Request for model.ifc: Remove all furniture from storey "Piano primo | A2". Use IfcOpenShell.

First a look at what the model holds.

```python
import ifcopenshell
import ifcopenshell.util.element

model = ifcopenshell.open("model.ifc")
print(model.schema)
storey = next(s for s in model.by_type("IfcBuildingStorey") if s.Name == "Piano primo | A2")
furniture = [e for e in ifcopenshell.util.element.get_decomposition(storey) if e.is_a("IfcFurnishingElement")]
seen = {}
for e in furniture:
    element_type = ifcopenshell.util.element.get_type(e)
    name = element_type.Name if element_type not in (None, e) else None
    seen[name] = seen.get(name, 0) + 1
for name, count in sorted(seen.items(), key=str):
    print(count, "x", name)
```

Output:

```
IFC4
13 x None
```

```python
import ifcopenshell
import ifcopenshell.api.root
import ifcopenshell.util.element

model = ifcopenshell.open("model.ifc")

storey = next(s for s in model.by_type("IfcBuildingStorey") if s.Name == "Piano primo | A2")
furniture = [e for e in ifcopenshell.util.element.get_decomposition(storey) if e.is_a("IfcFurnishingElement")]

for e in furniture:
    ifcopenshell.api.root.remove_product(model, product=e)
print(len(furniture), "removed")

model.write("model_edited.ifc")
```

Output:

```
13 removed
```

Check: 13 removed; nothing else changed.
